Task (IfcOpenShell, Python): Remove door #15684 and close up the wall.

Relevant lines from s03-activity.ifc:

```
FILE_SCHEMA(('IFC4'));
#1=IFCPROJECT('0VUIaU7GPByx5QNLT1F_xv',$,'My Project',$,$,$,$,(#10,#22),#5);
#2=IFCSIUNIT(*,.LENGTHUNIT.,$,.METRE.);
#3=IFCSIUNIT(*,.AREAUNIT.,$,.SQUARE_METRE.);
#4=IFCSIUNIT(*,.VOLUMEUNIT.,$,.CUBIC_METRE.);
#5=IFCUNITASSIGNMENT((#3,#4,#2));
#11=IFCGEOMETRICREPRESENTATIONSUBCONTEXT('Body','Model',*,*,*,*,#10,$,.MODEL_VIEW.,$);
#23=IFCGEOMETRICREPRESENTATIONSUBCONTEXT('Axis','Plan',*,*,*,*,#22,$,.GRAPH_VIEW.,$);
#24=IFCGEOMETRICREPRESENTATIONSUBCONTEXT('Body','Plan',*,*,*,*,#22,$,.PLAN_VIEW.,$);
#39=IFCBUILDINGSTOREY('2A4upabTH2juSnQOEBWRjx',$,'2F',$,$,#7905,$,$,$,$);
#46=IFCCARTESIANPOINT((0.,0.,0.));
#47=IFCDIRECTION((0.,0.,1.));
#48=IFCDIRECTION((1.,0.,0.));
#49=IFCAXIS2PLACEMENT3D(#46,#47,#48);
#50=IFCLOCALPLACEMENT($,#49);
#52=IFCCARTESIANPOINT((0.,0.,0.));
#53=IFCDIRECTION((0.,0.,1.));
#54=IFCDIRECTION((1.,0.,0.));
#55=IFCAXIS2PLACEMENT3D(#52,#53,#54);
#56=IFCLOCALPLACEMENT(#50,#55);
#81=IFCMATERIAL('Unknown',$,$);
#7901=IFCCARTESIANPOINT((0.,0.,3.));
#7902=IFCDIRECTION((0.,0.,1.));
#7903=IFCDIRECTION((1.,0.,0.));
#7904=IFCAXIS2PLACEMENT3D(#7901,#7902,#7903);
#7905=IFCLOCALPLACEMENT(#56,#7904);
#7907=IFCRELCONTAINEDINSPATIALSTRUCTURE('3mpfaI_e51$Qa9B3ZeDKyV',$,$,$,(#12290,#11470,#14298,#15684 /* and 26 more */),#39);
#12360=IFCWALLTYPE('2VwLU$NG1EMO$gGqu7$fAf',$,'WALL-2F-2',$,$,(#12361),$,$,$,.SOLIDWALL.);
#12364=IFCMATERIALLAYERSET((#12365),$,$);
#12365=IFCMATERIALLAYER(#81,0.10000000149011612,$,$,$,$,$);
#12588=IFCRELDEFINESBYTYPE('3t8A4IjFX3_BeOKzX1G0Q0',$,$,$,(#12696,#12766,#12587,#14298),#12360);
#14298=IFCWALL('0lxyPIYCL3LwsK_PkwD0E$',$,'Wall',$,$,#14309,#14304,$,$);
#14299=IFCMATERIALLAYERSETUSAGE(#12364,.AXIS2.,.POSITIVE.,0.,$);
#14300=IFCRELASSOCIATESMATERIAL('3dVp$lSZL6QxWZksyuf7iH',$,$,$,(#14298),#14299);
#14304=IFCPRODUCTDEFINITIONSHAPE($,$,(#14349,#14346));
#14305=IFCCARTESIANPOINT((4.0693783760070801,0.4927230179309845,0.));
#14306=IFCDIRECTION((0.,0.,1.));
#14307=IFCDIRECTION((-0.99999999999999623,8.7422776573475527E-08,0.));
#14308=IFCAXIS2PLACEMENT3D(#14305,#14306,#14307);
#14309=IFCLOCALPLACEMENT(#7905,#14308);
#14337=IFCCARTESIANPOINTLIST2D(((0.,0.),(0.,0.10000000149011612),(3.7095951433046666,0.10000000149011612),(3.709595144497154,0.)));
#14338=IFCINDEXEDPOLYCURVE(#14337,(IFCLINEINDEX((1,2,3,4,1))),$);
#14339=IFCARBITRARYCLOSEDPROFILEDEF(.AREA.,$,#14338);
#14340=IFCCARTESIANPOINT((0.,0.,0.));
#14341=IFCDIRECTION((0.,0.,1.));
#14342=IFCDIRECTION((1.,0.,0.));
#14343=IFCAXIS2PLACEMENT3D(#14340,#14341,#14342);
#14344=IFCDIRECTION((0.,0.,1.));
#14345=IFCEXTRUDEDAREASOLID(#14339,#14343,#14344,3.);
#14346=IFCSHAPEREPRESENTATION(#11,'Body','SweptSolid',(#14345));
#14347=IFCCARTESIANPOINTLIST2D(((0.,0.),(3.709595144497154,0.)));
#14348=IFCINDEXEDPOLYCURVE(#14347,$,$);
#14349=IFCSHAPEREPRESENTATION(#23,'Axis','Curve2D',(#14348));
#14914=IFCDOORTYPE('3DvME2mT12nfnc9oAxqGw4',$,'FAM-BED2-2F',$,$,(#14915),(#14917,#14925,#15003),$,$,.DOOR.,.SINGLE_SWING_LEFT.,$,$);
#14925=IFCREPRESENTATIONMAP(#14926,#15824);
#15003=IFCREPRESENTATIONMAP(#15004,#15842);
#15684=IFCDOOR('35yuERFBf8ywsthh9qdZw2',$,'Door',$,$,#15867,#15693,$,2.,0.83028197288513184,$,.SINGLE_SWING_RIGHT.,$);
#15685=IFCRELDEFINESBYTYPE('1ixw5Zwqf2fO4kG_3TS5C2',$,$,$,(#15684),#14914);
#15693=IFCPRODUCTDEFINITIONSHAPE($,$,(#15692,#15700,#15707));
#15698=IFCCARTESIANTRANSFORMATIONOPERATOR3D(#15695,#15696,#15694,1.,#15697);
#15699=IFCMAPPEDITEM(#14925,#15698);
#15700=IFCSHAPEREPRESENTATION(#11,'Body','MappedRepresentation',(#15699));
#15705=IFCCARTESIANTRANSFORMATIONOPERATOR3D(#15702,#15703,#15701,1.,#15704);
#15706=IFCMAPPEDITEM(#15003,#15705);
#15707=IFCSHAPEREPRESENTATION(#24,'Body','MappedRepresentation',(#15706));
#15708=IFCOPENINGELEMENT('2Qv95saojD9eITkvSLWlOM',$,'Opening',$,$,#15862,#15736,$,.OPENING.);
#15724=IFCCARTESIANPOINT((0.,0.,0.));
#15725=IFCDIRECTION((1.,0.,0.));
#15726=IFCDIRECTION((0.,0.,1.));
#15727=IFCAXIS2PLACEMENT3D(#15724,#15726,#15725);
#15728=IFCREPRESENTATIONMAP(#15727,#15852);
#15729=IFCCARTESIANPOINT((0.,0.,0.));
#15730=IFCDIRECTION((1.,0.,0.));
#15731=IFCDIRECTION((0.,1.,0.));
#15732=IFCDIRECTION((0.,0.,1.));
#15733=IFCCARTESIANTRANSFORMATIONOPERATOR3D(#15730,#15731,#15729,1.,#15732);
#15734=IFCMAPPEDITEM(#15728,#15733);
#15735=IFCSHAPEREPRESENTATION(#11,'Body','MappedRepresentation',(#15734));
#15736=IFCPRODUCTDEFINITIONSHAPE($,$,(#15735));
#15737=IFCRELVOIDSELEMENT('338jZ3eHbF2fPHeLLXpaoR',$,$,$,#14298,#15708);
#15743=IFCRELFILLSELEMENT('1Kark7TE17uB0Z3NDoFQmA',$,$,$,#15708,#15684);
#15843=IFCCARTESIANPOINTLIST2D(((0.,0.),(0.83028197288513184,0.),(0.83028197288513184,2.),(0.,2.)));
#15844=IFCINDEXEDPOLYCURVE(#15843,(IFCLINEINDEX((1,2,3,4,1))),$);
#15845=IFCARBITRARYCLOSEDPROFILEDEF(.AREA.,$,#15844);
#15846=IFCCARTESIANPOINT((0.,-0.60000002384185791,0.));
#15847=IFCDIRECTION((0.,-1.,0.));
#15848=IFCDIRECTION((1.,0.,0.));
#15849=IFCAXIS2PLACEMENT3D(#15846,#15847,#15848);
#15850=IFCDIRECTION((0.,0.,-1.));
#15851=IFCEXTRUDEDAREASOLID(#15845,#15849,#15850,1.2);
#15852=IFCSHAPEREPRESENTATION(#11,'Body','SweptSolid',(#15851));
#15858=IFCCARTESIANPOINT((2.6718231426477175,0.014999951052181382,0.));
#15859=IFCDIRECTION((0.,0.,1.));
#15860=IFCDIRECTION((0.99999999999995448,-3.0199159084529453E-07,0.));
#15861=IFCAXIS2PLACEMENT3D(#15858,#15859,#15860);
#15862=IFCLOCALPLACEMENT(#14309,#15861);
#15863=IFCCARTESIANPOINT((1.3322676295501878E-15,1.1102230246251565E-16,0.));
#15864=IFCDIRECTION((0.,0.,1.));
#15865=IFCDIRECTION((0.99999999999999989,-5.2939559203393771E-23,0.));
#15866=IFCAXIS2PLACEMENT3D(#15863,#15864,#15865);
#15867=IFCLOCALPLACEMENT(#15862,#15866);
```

```python
import ifcopenshell
import ifcopenshell.api.feature
import ifcopenshell.api.root
import ifcopenshell.geom
import ifcopenshell.util.shape

model = ifcopenshell.open("s03-activity.ifc")
settings = ifcopenshell.geom.settings()


def volume(element):
    """Net volume in cubic metres, openings subtracted."""
    shape = ifcopenshell.geom.create_shape(settings, element)
    return ifcopenshell.util.shape.get_volume(shape.geometry)


door = model.by_guid("35yuERFBf8ywsthh9qdZw2")
opening = door.FillsVoids[0].RelatingOpeningElement
wall = opening.VoidsElements[0].RelatingBuildingElement
before = volume(wall)

ifcopenshell.api.root.remove_product(model, product=door)
ifcopenshell.api.feature.remove_feature(model, feature=opening)

after = volume(wall)

print(f"wall volume {before:.3f} -> {after:.3f} m3")

model.write("s03-activity_rev.ifc")
```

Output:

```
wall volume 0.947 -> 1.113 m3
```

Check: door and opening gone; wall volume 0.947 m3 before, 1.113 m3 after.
